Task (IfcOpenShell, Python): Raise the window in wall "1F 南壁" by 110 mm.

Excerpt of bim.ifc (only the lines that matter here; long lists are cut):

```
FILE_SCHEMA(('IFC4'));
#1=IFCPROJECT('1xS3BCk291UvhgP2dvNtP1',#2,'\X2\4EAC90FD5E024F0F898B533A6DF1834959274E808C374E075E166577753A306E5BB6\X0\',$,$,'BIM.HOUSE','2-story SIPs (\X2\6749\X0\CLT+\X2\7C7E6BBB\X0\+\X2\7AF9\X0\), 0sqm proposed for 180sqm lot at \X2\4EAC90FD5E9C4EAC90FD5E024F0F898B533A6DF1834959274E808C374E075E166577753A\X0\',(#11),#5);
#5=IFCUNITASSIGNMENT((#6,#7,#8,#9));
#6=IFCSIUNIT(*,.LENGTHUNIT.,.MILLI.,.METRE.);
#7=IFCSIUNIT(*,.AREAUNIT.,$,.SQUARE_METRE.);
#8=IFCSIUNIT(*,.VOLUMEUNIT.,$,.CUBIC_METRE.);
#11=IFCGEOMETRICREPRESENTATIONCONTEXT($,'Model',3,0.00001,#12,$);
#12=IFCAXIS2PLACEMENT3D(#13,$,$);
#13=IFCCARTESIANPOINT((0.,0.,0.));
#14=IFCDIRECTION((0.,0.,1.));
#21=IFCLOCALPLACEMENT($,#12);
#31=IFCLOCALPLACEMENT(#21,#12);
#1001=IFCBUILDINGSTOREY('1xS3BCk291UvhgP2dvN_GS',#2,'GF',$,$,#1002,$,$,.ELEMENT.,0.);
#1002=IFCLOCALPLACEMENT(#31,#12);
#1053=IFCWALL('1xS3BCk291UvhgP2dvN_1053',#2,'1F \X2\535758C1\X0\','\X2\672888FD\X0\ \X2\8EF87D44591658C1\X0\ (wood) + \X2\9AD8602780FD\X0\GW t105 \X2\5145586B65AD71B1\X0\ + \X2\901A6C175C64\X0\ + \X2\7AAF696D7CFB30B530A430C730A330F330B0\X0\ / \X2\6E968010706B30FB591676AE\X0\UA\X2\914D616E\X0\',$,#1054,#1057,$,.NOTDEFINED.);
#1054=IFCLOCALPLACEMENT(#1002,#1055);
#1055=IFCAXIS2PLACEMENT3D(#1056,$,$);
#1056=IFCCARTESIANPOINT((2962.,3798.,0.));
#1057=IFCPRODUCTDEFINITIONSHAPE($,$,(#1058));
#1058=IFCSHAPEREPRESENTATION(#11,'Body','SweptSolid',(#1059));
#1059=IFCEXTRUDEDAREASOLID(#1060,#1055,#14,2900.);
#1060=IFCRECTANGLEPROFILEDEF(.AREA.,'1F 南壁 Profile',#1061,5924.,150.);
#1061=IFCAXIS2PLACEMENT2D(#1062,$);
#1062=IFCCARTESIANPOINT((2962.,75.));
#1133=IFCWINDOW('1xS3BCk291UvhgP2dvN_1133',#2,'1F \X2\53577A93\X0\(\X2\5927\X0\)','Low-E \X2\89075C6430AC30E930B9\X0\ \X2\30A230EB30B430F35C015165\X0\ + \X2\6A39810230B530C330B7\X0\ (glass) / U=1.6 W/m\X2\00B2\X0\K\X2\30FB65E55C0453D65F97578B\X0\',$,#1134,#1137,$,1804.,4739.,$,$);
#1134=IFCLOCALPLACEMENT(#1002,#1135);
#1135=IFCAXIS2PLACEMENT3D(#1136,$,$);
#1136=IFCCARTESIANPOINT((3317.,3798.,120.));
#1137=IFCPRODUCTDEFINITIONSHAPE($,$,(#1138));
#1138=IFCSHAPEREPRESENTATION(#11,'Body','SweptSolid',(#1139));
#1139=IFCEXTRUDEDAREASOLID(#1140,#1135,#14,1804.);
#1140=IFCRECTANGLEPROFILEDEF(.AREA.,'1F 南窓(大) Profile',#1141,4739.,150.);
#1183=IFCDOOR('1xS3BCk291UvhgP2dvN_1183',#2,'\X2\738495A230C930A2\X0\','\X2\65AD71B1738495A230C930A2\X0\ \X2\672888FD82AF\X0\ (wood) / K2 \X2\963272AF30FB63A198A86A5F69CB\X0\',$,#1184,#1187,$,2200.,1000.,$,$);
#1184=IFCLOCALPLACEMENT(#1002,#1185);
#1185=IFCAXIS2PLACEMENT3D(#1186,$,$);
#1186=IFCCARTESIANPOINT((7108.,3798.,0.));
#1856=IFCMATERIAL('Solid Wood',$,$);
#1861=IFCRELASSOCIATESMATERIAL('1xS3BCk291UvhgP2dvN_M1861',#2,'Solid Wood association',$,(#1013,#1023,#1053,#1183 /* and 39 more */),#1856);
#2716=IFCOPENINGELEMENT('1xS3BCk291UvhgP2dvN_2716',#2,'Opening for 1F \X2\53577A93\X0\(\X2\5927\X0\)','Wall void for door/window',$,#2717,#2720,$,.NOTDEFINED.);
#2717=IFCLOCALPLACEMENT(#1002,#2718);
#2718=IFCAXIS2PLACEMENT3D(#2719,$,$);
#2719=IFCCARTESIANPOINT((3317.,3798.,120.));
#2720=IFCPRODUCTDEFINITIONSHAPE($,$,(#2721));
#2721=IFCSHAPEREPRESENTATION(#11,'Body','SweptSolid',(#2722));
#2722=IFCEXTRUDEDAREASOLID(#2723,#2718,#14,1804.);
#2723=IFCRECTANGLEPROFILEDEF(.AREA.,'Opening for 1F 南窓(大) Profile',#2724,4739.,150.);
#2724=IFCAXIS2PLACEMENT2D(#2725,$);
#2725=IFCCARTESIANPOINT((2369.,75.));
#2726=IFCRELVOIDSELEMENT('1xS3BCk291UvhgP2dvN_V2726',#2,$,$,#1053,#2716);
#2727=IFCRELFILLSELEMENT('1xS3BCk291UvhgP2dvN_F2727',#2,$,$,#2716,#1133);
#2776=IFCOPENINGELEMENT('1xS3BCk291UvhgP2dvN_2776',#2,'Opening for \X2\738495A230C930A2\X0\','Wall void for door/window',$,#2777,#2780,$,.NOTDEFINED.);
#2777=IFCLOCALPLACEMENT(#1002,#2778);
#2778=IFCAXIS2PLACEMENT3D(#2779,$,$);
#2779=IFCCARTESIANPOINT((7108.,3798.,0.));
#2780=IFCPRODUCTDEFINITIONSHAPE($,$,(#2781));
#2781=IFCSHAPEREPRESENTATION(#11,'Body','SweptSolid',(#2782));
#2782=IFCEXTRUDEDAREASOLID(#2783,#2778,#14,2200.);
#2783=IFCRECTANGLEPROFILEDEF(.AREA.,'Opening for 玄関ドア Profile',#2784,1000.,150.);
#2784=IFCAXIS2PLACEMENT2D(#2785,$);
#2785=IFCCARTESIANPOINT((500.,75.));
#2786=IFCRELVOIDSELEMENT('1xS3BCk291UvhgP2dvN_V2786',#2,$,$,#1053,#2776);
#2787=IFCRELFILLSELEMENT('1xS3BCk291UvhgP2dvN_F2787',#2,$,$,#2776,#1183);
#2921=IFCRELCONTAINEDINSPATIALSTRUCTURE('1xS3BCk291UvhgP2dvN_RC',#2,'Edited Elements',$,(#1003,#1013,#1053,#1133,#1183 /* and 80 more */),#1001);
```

```python
import numpy as np
import ifcopenshell
import ifcopenshell.api.geometry
import ifcopenshell.util.placement
import ifcopenshell.util.unit

model = ifcopenshell.open("bim.ifc")
unit_scale = ifcopenshell.util.unit.calculate_unit_scale(model)

window = model.by_id(1133)
opening = window.FillsVoids[0].RelatingOpeningElement
dz = 0.11 / unit_scale

shift = np.array([0.0, 0.0, dz])
# The window is not placed relative to its opening, so move both.
for product in (opening, window):
    matrix = ifcopenshell.util.placement.get_local_placement(product.ObjectPlacement)
    matrix[:3, 3] += shift
    ifcopenshell.api.geometry.edit_object_placement(model, product=product, matrix=matrix, is_si=False)

print(f"moved by {dz * unit_scale:+.3f} m")

model.write("bim_rev.ifc")
```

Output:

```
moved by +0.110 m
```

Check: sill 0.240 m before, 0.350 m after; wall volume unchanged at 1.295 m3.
